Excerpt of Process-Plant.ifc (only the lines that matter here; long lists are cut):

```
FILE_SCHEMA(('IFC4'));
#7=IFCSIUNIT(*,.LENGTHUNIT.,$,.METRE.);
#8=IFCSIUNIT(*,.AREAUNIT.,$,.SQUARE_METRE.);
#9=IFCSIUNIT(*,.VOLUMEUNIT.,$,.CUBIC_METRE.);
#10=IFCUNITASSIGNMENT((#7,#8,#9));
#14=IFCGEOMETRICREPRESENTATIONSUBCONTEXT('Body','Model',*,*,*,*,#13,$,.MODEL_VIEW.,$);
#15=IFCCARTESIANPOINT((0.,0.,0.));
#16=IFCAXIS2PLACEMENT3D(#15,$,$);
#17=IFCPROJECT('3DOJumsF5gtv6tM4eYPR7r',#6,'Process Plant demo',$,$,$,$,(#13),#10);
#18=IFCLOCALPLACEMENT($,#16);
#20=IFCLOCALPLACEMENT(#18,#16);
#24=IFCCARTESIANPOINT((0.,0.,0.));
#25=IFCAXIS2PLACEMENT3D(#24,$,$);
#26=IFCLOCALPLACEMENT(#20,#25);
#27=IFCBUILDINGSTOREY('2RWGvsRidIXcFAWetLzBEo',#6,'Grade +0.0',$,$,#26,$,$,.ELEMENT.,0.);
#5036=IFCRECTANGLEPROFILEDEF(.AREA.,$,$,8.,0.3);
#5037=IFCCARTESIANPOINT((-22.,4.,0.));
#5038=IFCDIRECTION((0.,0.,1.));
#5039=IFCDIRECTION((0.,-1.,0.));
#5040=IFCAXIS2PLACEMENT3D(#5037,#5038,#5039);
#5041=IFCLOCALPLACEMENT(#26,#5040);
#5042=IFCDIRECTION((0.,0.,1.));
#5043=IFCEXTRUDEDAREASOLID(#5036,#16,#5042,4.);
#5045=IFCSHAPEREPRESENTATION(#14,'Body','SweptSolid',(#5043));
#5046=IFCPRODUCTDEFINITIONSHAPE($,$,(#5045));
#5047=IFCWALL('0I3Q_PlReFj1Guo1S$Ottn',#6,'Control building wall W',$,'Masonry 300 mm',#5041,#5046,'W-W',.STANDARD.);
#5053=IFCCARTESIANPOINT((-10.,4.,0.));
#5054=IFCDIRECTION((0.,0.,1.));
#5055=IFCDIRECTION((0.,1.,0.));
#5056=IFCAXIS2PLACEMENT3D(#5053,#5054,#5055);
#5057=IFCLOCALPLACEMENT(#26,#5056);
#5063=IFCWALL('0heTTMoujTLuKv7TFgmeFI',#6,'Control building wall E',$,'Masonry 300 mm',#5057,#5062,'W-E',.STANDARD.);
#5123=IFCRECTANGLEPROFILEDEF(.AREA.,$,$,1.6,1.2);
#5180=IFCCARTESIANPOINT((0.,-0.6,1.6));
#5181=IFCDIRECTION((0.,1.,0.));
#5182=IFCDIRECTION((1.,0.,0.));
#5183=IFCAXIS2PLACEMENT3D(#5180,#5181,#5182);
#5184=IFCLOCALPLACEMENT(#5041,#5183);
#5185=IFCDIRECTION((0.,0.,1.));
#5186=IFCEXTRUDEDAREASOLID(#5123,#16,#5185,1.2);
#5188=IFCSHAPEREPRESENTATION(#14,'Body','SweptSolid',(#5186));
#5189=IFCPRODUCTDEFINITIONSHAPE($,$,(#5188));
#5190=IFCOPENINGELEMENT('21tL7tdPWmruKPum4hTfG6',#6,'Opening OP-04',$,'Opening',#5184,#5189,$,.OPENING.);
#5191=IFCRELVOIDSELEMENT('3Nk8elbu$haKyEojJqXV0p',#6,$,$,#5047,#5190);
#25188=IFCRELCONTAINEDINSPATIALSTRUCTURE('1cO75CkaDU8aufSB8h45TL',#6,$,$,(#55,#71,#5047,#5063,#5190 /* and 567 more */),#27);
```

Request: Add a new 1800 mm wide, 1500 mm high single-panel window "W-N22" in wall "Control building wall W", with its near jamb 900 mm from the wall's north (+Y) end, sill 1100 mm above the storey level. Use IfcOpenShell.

```python
import numpy as np
import ifcopenshell
import ifcopenshell.api.feature
import ifcopenshell.api.geometry
import ifcopenshell.api.root
import ifcopenshell.api.spatial
import ifcopenshell.geom
import ifcopenshell.util.element
import ifcopenshell.util.placement
import ifcopenshell.util.representation
import ifcopenshell.util.shape
import ifcopenshell.util.unit

model = ifcopenshell.open("Process-Plant.ifc")
unit_scale = ifcopenshell.util.unit.calculate_unit_scale(model)
settings = ifcopenshell.geom.settings()


def volume(element):
    """Net volume in cubic metres, openings subtracted."""
    shape = ifcopenshell.geom.create_shape(settings, element)
    return ifcopenshell.util.shape.get_volume(shape.geometry)


wall = model.by_guid("0I3Q_PlReFj1Guo1S$Ottn")
storey = ifcopenshell.util.element.get_container(wall, ifc_class="IfcBuildingStorey")
context = ifcopenshell.util.representation.get_context(model, "Model", "Body", "MODEL_VIEW")
before = volume(wall)

width, height, from_end, sill = 1.8, 1.5, 0.9, 1.1  # metres

# The wall runs along its own X axis, and the end named is its -X end.
wall_shape = ifcopenshell.geom.create_shape(settings, wall)
x, y, z = ifcopenshell.util.shape.get_vertices(wall_shape.geometry).T
start = x.min() + from_end
face, thickness = float(y.min()), float(y.max() - y.min())
wall_matrix = ifcopenshell.util.placement.get_local_placement(wall.ObjectPlacement)
level = ifcopenshell.util.placement.get_local_placement(storey.ObjectPlacement)[2, 3]


def in_wall(x, y):
    """Placement at x, y metres in the wall's axes, at sill height."""
    matrix = wall_matrix.copy()
    matrix[:, 3] = wall_matrix @ np.array([x / unit_scale, y / unit_scale, 0.0, 1.0])
    matrix[2, 3] = level + sill / unit_scale
    return matrix


# Opening: a box that overshoots both wall faces by 50 mm.
opening = ifcopenshell.api.root.create_entity(model, ifc_class="IfcOpeningElement", predefined_type="OPENING")
box = ifcopenshell.api.geometry.add_wall_representation(
    model, context=context, length=width, height=height, thickness=thickness + 0.1
)
ifcopenshell.api.geometry.assign_representation(model, product=opening, representation=box)
ifcopenshell.api.geometry.edit_object_placement(model, product=opening, matrix=in_wall(start, face - 0.05), is_si=False)
ifcopenshell.api.feature.add_feature(model, feature=opening, element=wall)

window = ifcopenshell.api.root.create_entity(model, ifc_class="IfcWindow", name="W-N22", predefined_type="WINDOW")
window.OverallWidth, window.OverallHeight = width / unit_scale, height / unit_scale
window.PartitioningType = "SINGLE_PANEL"
body = ifcopenshell.api.geometry.add_window_representation(
    model,
    context=context,
    overall_width=window.OverallWidth,
    overall_height=window.OverallHeight,
    partition_type="SINGLE_PANEL",
)
ifcopenshell.api.geometry.assign_representation(model, product=window, representation=body)
ifcopenshell.api.spatial.assign_container(model, products=[window], relating_structure=storey)
ifcopenshell.api.feature.add_filling(model, opening=opening, element=window)

# Centre the window in the wall's thickness.
ifcopenshell.api.geometry.edit_object_placement(model, product=window, matrix=in_wall(start, face), is_si=False)
window_shape = ifcopenshell.geom.create_shape(settings, window)
depth = ifcopenshell.util.shape.get_vertices(window_shape.geometry)[:, 1]
offset = face + thickness / 2 - (depth.min() + depth.max()) / 2
ifcopenshell.api.geometry.edit_object_placement(model, product=window, matrix=in_wall(start, offset), is_si=False)

after = volume(wall)

print(f"wall volume {before:.3f} -> {after:.3f} m3")

model.write("Process-Plant_edited.ifc")
```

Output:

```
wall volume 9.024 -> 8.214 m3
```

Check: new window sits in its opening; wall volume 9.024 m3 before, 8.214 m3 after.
